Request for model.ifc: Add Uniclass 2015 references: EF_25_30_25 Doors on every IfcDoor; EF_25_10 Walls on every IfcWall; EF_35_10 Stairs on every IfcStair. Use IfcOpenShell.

First a look at what the model holds.

```python
import ifcopenshell

model = ifcopenshell.open("model.ifc")
print(model.schema)
print("classifications:", [c.Name for c in model.by_type("IfcClassification")])
for ifc_class in ("IfcDoor", "IfcRoof", "IfcStair", "IfcWall", "IfcWindow"):
    print(ifc_class, len(model.by_type(ifc_class)))
```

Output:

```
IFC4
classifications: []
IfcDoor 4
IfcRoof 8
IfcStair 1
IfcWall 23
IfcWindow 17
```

```python
import ifcopenshell
import ifcopenshell.api.classification

model = ifcopenshell.open("model.ifc")

system = ifcopenshell.api.classification.add_classification(model, classification="Uniclass 2015")

codes = {
    "IfcDoor": ("EF_25_30_25", "Doors"),
    "IfcWall": ("EF_25_10", "Walls"),
    "IfcStair": ("EF_35_10", "Stairs"),
}
for ifc_class, (code, name) in codes.items():
    products = model.by_type(ifc_class)
    ifcopenshell.api.classification.add_reference(
        model, products=products, classification=system, identification=code, name=name
    )
    print(code, len(products))

model.write("model_updated.ifc")
```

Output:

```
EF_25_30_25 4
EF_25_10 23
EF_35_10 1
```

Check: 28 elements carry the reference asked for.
